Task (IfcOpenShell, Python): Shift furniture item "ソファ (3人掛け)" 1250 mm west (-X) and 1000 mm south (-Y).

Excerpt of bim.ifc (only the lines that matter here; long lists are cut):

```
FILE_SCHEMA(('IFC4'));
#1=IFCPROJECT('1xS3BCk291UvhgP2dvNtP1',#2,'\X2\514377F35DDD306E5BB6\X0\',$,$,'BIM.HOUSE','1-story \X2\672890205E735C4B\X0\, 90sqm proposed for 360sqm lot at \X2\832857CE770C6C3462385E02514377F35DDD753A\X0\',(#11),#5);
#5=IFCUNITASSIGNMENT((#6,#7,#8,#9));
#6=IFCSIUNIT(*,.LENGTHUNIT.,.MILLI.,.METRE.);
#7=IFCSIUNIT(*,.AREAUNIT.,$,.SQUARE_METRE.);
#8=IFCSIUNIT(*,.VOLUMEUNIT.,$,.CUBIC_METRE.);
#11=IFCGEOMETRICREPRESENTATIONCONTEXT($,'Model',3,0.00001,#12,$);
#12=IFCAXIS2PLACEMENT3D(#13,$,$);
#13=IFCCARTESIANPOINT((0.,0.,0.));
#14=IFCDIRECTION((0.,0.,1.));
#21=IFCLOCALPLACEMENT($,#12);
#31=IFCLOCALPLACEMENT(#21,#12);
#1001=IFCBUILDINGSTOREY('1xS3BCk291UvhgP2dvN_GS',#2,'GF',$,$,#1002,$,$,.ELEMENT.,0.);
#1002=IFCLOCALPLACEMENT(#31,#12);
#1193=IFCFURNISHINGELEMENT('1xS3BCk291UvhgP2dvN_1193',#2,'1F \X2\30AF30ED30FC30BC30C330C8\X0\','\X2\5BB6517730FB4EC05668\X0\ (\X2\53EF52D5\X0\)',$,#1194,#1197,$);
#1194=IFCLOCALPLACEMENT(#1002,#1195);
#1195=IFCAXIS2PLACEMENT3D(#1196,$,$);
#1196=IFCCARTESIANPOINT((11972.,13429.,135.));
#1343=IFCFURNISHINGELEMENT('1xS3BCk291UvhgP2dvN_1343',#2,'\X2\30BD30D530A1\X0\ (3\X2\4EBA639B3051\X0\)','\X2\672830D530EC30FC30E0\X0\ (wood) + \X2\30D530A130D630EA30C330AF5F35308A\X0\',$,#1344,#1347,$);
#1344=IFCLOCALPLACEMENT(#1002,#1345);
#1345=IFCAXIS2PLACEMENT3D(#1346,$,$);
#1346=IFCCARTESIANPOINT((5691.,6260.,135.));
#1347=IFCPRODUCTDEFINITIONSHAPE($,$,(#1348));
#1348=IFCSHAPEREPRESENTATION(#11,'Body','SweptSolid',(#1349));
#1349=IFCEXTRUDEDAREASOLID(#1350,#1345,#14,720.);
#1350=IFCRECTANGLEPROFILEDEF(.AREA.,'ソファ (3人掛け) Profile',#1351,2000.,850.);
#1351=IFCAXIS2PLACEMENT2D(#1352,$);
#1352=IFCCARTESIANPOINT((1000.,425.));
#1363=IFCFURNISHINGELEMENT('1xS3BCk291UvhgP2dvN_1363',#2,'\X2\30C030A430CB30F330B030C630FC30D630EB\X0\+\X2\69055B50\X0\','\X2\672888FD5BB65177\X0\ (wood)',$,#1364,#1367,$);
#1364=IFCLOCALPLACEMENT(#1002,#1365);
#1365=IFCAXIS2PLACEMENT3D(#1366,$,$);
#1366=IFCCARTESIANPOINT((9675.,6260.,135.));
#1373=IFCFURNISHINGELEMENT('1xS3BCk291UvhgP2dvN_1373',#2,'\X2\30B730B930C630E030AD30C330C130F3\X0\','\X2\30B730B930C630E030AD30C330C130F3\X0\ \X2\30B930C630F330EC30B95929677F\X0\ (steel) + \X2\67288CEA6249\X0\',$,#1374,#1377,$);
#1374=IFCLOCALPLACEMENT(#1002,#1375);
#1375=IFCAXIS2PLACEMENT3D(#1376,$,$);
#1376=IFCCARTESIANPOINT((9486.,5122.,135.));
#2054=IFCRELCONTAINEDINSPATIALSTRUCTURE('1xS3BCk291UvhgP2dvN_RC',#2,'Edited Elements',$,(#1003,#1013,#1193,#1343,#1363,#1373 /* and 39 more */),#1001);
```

```python
import ifcopenshell
import ifcopenshell.api.geometry
import ifcopenshell.util.placement
import ifcopenshell.util.unit

model = ifcopenshell.open("bim.ifc")
unit_scale = ifcopenshell.util.unit.calculate_unit_scale(model)

item = model.by_guid("1xS3BCk291UvhgP2dvN_1343")
matrix = ifcopenshell.util.placement.get_local_placement(item.ObjectPlacement)
matrix[0, 3] -= 1.25 / unit_scale
matrix[1, 3] -= 1 / unit_scale
ifcopenshell.api.geometry.edit_object_placement(model, product=item, matrix=matrix, is_si=False)

print(ifcopenshell.util.placement.get_local_placement(item.ObjectPlacement).round(3) + 0.0)

model.write("bim_rev.ifc")
```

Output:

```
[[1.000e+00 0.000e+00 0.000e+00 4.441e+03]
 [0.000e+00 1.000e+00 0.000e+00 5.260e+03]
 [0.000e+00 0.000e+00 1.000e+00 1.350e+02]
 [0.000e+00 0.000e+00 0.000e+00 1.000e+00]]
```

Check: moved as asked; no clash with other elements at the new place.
